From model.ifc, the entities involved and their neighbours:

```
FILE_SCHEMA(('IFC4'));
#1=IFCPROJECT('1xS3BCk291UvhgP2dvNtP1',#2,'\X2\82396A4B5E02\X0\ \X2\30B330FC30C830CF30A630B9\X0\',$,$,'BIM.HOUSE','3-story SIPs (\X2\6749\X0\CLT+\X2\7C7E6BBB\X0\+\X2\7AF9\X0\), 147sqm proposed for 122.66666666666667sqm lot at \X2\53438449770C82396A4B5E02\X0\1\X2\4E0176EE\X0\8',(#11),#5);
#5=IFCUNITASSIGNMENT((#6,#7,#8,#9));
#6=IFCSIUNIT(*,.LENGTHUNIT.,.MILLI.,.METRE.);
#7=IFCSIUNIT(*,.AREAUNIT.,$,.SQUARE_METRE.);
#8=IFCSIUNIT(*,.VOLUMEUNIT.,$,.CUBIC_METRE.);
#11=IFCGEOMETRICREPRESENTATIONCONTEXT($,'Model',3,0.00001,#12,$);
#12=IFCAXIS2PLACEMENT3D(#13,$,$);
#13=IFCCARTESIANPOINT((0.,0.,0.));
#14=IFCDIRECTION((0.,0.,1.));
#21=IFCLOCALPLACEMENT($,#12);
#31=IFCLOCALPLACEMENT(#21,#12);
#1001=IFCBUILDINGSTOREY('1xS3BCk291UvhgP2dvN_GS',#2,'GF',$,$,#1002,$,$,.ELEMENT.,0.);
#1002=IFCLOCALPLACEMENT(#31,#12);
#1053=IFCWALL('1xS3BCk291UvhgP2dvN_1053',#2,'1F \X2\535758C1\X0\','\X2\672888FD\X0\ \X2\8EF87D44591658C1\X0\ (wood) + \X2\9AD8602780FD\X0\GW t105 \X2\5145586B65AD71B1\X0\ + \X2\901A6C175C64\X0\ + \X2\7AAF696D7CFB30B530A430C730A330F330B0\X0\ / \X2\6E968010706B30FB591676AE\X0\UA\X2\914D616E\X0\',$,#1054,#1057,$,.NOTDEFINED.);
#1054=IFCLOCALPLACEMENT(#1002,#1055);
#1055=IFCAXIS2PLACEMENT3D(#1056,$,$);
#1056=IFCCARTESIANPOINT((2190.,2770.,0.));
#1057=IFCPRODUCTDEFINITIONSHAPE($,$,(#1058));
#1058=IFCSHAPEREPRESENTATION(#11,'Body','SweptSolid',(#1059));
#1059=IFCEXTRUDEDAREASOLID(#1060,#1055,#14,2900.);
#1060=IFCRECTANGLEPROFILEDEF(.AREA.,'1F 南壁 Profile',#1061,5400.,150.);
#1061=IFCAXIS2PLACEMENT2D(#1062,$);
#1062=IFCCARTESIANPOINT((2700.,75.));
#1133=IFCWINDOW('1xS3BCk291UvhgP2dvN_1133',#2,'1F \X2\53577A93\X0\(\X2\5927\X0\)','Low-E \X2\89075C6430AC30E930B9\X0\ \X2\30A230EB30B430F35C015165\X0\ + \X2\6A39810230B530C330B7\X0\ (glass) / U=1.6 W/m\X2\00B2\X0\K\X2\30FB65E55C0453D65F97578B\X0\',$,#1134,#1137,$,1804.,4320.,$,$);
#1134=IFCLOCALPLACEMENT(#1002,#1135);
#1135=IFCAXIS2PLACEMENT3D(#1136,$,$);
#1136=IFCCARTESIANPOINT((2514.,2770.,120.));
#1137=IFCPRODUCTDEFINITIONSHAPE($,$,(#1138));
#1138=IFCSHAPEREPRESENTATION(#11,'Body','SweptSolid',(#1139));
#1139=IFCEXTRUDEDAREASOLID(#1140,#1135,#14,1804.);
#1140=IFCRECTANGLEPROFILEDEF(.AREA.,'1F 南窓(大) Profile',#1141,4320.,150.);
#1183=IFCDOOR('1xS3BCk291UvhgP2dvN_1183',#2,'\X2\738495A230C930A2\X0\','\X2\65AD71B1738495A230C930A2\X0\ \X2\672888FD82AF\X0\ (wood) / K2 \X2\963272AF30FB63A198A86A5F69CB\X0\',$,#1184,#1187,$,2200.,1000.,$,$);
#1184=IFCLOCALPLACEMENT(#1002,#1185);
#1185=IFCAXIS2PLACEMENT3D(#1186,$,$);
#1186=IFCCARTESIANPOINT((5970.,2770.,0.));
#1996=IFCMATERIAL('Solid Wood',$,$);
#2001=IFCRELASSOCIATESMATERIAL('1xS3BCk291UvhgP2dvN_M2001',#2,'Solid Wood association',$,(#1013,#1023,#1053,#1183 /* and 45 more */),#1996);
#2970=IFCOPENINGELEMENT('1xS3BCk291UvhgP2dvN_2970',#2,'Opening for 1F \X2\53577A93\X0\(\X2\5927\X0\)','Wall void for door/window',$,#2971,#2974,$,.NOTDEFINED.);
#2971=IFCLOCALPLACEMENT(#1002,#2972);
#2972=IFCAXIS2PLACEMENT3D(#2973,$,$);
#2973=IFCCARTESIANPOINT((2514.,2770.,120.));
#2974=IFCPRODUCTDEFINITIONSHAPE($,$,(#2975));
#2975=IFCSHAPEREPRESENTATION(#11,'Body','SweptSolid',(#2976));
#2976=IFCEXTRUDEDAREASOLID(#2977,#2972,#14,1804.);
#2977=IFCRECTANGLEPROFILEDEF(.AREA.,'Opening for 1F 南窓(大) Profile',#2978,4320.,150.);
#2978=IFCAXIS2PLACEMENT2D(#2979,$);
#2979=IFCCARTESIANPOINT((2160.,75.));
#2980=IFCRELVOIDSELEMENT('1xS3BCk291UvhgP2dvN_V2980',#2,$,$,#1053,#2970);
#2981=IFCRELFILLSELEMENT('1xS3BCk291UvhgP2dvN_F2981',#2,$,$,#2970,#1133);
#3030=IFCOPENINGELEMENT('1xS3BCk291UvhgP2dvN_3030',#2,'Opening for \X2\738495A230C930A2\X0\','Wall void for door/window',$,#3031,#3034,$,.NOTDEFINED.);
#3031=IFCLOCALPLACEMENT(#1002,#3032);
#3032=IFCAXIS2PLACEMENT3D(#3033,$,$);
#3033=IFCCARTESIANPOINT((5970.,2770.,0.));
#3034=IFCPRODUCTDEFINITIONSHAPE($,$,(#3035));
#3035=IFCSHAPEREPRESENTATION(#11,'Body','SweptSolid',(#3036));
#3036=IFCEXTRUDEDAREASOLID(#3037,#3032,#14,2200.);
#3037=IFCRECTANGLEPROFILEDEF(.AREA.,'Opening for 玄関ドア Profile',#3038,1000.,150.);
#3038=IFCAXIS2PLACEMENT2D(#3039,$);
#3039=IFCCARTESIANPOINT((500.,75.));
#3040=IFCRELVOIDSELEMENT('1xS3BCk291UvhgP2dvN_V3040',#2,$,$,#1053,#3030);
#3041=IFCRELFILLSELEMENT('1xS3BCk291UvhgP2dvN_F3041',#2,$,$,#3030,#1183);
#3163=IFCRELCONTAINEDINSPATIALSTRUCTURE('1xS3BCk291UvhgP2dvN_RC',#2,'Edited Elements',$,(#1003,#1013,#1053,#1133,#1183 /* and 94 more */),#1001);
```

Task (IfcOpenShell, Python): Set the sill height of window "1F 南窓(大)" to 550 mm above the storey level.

```python
import numpy as np
import ifcopenshell
import ifcopenshell.api.geometry
import ifcopenshell.geom
import ifcopenshell.util.element
import ifcopenshell.util.placement
import ifcopenshell.util.shape
import ifcopenshell.util.unit

model = ifcopenshell.open("model.ifc")
unit_scale = ifcopenshell.util.unit.calculate_unit_scale(model)

window = model.by_id(1133)
opening = window.FillsVoids[0].RelatingOpeningElement
storey = ifcopenshell.util.element.get_container(window, ifc_class="IfcBuildingStorey")
level = ifcopenshell.util.placement.get_local_placement(storey.ObjectPlacement)[2, 3]

# The opening's origin need not be at the sill, so measure its lowest point.
shape = ifcopenshell.geom.create_shape(ifcopenshell.geom.settings(), opening)
bottom = ifcopenshell.util.shape.get_shape_bottom_elevation(shape, shape.geometry) / unit_scale
dz = level + 0.55 / unit_scale - bottom

shift = np.array([0.0, 0.0, dz])
# The window is not placed relative to its opening, so move both.
for product in (opening, window):
    matrix = ifcopenshell.util.placement.get_local_placement(product.ObjectPlacement)
    matrix[:3, 3] += shift
    ifcopenshell.api.geometry.edit_object_placement(model, product=product, matrix=matrix, is_si=False)

print(f"moved by {dz * unit_scale:+.3f} m")

model.write("model_updated.ifc")
```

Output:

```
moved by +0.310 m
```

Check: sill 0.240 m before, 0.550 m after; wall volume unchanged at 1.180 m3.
